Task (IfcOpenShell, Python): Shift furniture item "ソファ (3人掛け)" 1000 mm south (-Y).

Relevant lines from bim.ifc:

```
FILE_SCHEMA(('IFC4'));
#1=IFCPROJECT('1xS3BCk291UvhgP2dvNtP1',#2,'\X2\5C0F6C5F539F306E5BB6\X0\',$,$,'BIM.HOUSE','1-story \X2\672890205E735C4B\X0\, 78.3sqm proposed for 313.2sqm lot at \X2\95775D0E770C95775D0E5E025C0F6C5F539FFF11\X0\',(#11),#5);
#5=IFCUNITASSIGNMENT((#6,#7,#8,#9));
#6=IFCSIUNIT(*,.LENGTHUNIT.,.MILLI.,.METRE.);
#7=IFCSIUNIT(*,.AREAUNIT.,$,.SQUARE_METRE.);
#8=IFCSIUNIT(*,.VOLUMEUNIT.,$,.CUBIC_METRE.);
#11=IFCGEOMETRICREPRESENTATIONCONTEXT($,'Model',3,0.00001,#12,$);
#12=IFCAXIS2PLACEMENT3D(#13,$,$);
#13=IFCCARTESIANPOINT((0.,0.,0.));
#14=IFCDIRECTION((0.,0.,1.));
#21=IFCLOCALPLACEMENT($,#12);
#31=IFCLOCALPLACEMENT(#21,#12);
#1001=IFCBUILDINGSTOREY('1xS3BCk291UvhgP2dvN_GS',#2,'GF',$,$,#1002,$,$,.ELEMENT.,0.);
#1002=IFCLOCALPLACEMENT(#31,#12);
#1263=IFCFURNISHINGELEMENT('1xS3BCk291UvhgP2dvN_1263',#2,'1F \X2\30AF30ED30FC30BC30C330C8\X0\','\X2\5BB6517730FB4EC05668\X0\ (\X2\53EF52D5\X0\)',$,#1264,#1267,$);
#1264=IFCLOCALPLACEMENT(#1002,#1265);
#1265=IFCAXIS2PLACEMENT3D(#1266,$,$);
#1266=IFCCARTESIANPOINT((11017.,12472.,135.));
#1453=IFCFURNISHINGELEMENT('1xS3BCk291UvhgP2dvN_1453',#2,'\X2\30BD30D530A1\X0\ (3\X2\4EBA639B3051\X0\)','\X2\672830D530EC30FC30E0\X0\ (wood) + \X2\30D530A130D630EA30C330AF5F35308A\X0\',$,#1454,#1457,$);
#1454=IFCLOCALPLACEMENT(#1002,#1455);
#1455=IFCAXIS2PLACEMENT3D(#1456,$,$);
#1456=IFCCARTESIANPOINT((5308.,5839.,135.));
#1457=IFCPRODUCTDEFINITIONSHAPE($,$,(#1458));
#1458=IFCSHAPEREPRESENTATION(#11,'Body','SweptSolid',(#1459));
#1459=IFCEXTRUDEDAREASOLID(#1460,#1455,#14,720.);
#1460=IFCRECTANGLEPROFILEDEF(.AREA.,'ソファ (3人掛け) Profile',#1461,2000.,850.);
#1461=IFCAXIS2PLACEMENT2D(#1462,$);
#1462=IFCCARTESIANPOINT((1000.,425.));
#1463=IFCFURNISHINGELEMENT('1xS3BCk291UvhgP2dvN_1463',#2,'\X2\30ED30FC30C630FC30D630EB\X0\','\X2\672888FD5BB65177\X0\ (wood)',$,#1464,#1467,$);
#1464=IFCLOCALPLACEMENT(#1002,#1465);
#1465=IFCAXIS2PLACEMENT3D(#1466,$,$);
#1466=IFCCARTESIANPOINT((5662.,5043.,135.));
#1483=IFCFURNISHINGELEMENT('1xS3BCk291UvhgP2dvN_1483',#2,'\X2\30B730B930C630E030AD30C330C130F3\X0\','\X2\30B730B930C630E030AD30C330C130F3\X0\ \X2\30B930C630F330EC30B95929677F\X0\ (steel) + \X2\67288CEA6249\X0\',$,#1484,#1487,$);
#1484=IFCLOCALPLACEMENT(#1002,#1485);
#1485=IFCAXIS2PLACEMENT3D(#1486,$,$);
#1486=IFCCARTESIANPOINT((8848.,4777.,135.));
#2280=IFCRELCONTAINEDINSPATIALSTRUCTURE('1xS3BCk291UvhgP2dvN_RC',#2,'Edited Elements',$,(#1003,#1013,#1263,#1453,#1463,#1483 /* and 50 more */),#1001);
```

```python
import ifcopenshell
import ifcopenshell.api.geometry
import ifcopenshell.util.placement
import ifcopenshell.util.unit

model = ifcopenshell.open("bim.ifc")
unit_scale = ifcopenshell.util.unit.calculate_unit_scale(model)

item = model.by_id(1453)
matrix = ifcopenshell.util.placement.get_local_placement(item.ObjectPlacement)
matrix[1, 3] -= 1 / unit_scale
ifcopenshell.api.geometry.edit_object_placement(model, product=item, matrix=matrix, is_si=False)

print(ifcopenshell.util.placement.get_local_placement(item.ObjectPlacement).round(3) + 0.0)

model.write("bim-out.ifc")
```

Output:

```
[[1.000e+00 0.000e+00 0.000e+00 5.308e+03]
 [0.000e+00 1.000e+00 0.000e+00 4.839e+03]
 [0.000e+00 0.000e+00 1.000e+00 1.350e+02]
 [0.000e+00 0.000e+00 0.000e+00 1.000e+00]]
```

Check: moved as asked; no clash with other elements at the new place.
